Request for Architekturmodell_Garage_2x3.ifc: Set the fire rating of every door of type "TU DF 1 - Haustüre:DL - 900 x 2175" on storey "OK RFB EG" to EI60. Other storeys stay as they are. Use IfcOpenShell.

First a look at what the model holds.

```python
import ifcopenshell
import ifcopenshell.util.element

model = ifcopenshell.open("Architekturmodell_Garage_2x3.ifc")
print(model.schema)
storey = next(s for s in model.by_type("IfcBuildingStorey") if s.Name == "OK RFB EG")
doors = [e for e in ifcopenshell.util.element.get_decomposition(storey) if e.is_a("IfcDoor")]
seen = {}
for e in doors:
    element_type = ifcopenshell.util.element.get_type(e)
    key = (element_type.Name if element_type != e and element_type else None, ifcopenshell.util.element.get_pset(e, "Pset_DoorCommon", "FireRating"))
    seen[key] = seen.get(key, 0) + 1
for (name, value), count in sorted(seen.items(), key=str):
    print(count, "x", name, "|", value)
```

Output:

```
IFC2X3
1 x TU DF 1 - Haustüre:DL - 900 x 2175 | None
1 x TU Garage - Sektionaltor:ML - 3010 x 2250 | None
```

```python
import ifcopenshell
import ifcopenshell.api.pset
import ifcopenshell.util.element

model = ifcopenshell.open("Architekturmodell_Garage_2x3.ifc")

storey = next(s for s in model.by_type("IfcBuildingStorey") if s.Name == "OK RFB EG")
doors = [e for e in ifcopenshell.util.element.get_decomposition(storey) if e.is_a("IfcDoor")]

count = 0
for e in doors:
    element_type = ifcopenshell.util.element.get_type(e)
    if element_type in (None, e) or element_type.Name != "TU DF 1 - Haustüre:DL - 900 x 2175":
        continue
    # add_pset returns the element's existing set when there is one.
    pset = ifcopenshell.api.pset.add_pset(model, product=e, name="Pset_DoorCommon")
    ifcopenshell.api.pset.edit_pset(model, pset=pset, properties={"FireRating": "EI60"})
    count += 1

print(count, "doors updated")

model.write("Architekturmodell_Garage_2x3_v2.ifc")
```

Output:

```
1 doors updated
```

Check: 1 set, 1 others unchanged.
